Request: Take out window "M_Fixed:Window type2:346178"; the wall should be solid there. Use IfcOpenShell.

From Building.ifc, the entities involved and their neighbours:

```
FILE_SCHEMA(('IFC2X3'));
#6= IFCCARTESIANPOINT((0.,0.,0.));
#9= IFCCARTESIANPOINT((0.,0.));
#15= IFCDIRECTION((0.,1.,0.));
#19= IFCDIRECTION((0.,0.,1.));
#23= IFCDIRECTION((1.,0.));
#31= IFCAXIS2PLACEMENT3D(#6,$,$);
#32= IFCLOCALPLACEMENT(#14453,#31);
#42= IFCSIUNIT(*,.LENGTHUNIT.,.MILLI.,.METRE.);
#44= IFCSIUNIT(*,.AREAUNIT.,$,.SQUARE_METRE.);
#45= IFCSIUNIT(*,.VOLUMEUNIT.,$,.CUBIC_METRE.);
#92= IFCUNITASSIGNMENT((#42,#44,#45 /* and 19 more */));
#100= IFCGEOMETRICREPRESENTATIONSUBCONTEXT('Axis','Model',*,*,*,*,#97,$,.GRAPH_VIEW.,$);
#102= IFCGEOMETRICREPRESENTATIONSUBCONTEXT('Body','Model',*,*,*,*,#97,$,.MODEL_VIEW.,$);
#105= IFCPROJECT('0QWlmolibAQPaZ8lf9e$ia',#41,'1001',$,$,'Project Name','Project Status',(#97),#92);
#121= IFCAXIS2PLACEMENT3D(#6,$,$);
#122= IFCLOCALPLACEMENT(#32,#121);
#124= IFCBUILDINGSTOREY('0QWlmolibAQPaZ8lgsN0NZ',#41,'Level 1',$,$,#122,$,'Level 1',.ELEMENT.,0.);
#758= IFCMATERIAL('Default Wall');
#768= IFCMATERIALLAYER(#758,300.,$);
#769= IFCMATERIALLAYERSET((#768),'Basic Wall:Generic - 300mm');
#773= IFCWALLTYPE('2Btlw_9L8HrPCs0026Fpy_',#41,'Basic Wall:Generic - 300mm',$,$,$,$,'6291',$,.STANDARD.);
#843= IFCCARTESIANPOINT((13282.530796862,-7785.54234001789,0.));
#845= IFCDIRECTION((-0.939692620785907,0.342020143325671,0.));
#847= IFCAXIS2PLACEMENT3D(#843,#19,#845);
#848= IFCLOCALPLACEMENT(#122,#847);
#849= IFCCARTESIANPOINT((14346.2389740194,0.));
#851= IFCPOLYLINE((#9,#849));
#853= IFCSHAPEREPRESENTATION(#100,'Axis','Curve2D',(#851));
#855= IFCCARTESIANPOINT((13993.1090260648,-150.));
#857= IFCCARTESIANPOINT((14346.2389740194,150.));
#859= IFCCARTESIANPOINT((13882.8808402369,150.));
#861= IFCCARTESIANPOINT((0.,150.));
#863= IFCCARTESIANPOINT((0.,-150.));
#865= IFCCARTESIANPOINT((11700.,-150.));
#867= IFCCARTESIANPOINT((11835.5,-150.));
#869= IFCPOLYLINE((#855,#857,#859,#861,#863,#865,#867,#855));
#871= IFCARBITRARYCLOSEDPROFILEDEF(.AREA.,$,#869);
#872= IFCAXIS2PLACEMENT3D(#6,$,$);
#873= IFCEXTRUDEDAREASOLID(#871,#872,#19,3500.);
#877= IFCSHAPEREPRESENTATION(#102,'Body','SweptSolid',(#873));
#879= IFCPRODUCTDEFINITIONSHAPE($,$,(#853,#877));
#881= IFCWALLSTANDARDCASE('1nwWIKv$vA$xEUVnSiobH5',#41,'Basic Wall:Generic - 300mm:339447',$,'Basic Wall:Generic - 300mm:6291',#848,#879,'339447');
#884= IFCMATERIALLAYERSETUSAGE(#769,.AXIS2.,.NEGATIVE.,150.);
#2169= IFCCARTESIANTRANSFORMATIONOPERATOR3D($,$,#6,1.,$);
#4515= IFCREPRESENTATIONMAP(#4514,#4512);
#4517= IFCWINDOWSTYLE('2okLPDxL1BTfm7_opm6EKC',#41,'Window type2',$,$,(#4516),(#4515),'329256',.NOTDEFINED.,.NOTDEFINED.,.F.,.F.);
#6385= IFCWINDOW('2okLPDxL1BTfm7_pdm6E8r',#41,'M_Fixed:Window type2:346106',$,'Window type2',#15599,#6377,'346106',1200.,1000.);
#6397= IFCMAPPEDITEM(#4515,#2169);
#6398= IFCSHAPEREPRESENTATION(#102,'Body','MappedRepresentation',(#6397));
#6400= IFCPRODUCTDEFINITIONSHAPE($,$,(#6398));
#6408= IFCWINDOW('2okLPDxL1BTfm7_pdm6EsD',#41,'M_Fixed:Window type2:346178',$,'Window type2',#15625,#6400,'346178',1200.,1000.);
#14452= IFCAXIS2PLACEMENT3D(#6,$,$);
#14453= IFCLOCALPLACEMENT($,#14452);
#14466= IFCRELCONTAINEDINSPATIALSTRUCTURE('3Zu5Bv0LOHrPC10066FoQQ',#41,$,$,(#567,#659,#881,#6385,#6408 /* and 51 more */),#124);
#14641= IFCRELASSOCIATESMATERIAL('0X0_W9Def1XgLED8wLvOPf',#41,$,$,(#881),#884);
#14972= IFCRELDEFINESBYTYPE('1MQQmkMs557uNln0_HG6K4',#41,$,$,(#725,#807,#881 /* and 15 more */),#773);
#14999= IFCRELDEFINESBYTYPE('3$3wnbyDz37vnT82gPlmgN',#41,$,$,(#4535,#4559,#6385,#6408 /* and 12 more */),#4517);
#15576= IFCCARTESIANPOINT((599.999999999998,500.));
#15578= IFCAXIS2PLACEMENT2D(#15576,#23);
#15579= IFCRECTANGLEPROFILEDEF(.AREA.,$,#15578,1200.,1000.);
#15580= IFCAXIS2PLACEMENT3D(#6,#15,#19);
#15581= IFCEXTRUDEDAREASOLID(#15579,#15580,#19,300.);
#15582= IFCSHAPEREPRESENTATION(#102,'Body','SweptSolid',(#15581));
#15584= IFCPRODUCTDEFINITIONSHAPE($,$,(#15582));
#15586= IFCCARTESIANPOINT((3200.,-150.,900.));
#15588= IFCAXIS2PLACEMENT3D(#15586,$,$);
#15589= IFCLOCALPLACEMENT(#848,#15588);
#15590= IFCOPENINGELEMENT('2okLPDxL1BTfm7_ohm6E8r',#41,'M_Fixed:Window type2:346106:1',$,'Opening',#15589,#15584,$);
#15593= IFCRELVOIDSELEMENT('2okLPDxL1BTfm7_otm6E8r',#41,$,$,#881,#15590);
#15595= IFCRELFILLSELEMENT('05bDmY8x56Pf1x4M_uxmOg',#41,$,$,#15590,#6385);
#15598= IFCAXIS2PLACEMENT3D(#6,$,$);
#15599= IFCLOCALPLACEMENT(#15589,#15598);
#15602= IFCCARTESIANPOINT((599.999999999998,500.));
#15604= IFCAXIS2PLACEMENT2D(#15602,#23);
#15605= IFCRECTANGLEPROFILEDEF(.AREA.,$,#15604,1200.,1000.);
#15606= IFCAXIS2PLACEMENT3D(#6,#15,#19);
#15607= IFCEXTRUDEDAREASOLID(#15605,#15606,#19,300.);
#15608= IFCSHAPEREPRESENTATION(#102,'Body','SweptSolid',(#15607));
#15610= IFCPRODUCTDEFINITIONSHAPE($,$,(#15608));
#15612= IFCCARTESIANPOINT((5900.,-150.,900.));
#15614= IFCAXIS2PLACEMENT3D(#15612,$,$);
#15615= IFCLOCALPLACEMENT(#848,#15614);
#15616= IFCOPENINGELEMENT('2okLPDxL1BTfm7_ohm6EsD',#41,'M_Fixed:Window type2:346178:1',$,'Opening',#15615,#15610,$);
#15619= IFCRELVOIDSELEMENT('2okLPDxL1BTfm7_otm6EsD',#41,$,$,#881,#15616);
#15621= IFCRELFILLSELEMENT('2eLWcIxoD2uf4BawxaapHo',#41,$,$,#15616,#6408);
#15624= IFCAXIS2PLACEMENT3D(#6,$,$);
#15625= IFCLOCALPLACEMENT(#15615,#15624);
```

```python
import ifcopenshell
import ifcopenshell.api.feature
import ifcopenshell.api.root
import ifcopenshell.geom
import ifcopenshell.util.shape

model = ifcopenshell.open("Building.ifc")
settings = ifcopenshell.geom.settings()


def volume(element):
    """Net volume in cubic metres, openings subtracted."""
    shape = ifcopenshell.geom.create_shape(settings, element)
    return ifcopenshell.util.shape.get_volume(shape.geometry)


window = model.by_id(6408)
opening = window.FillsVoids[0].RelatingOpeningElement
wall = opening.VoidsElements[0].RelatingBuildingElement
before = volume(wall)

ifcopenshell.api.root.remove_product(model, product=window)
ifcopenshell.api.feature.remove_feature(model, feature=opening)

after = volume(wall)

print(f"wall volume {before:.3f} -> {after:.3f} m3")

model.write("Building_v2.ifc")
```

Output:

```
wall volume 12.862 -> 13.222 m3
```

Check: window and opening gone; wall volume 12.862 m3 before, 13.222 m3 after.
